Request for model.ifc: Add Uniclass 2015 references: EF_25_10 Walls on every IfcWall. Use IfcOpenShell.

First a look at what the model holds.

```python
import ifcopenshell

model = ifcopenshell.open("model.ifc")
print(model.schema)
print("classifications:", [c.Name for c in model.by_type("IfcClassification")])
for ifc_class in ("IfcDoor", "IfcRoof", "IfcStair", "IfcWall", "IfcWindow"):
    print(ifc_class, len(model.by_type(ifc_class)))
```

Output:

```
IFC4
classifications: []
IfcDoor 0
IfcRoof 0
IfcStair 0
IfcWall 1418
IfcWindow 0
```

```python
import ifcopenshell
import ifcopenshell.api.classification

model = ifcopenshell.open("model.ifc")

system = ifcopenshell.api.classification.add_classification(model, classification="Uniclass 2015")

codes = {
    "IfcWall": ("EF_25_10", "Walls"),
}
for ifc_class, (code, name) in codes.items():
    products = model.by_type(ifc_class)
    ifcopenshell.api.classification.add_reference(
        model, products=products, classification=system, identification=code, name=name
    )
    print(code, len(products))

model.write("model_rev.ifc")
```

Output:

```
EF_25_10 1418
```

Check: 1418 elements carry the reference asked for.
